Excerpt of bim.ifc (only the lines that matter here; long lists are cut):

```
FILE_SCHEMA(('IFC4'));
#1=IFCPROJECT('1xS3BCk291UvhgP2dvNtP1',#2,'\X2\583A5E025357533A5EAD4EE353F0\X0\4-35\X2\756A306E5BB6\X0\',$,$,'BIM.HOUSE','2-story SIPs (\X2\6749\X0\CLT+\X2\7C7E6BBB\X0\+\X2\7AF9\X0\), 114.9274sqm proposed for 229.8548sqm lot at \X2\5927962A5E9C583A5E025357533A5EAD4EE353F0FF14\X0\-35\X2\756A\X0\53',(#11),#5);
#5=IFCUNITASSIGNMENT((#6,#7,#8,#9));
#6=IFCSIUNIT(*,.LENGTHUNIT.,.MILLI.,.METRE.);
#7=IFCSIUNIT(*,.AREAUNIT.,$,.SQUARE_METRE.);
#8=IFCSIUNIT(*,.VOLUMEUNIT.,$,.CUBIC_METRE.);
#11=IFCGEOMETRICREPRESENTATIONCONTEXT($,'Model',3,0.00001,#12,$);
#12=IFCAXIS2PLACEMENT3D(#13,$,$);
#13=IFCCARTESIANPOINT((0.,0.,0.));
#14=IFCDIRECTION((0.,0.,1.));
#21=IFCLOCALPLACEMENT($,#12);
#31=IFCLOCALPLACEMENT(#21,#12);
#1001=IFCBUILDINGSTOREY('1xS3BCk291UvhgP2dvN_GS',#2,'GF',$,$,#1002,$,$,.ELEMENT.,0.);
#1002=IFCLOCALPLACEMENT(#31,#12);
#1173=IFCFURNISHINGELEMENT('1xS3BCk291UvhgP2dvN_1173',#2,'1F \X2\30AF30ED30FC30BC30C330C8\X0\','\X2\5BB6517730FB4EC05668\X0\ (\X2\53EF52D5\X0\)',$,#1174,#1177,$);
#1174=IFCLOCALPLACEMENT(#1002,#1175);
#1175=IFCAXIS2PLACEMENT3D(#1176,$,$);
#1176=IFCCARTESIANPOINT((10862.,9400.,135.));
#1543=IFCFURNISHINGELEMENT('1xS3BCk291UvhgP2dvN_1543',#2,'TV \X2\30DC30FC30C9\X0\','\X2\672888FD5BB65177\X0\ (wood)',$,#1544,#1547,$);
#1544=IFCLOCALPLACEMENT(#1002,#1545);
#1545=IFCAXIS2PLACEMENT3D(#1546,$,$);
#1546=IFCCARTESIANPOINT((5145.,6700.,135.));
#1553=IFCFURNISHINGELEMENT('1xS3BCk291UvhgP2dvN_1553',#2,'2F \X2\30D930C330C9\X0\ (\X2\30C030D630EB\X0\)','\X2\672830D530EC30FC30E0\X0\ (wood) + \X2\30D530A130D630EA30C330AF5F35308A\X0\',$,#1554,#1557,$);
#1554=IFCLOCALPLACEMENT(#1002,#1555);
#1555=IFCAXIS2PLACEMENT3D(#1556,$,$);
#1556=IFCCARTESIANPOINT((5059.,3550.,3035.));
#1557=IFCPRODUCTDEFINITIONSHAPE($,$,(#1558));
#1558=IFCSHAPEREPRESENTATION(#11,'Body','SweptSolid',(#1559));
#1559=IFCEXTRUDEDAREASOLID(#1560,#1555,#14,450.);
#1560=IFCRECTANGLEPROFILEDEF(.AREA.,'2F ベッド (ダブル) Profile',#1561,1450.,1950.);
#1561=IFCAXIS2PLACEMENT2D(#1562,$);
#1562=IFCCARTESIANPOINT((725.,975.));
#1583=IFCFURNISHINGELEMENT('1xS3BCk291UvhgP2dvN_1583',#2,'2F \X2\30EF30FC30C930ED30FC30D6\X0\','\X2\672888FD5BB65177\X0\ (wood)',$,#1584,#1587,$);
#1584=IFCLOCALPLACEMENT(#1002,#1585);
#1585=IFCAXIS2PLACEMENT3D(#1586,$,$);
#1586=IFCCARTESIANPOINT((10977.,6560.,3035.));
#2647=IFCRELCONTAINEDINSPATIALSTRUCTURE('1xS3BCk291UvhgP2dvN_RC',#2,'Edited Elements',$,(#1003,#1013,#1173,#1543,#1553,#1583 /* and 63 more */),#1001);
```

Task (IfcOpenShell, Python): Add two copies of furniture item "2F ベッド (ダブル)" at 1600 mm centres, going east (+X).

```python
import numpy as np
import ifcopenshell
import ifcopenshell.api.geometry
import ifcopenshell.api.root
import ifcopenshell.util.element
import ifcopenshell.util.placement

model = ifcopenshell.open("bim.ifc")


def reuse_history(source, copy):
    """copy_class also copies each property set's owner history, people and application; keep the originals."""
    for rel in copy.IsDefinedBy:
        if rel.is_a("IfcRelDefinesByProperties") and (history := rel.RelatingPropertyDefinition.OwnerHistory):
            rel.RelatingPropertyDefinition.OwnerHistory = source.OwnerHistory
            ifcopenshell.util.element.remove_deep2(model, history)


source = model.by_guid("1xS3BCk291UvhgP2dvN_1553")
base = ifcopenshell.util.placement.get_local_placement(source.ObjectPlacement)
step = np.array([1.0, 0.0, 0.0]) * 1600.0

for i in range(1, 3):
    copy = ifcopenshell.api.root.copy_class(model, product=source)
    copy.Representation = ifcopenshell.util.element.copy_deep(
        model, source.Representation, exclude=["IfcGeometricRepresentationContext", "IfcRepresentationMap"]
    )
    reuse_history(source, copy)
    matrix = base.copy()
    matrix[:3, 3] += i * step
    print("added at", matrix[:3, 3].round(3) + 0.0)
    ifcopenshell.api.geometry.edit_object_placement(model, product=copy, matrix=matrix, is_si=False)

model.write("bim_rev.ifc")
```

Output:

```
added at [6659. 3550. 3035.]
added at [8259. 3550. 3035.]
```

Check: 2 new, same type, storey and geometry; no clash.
